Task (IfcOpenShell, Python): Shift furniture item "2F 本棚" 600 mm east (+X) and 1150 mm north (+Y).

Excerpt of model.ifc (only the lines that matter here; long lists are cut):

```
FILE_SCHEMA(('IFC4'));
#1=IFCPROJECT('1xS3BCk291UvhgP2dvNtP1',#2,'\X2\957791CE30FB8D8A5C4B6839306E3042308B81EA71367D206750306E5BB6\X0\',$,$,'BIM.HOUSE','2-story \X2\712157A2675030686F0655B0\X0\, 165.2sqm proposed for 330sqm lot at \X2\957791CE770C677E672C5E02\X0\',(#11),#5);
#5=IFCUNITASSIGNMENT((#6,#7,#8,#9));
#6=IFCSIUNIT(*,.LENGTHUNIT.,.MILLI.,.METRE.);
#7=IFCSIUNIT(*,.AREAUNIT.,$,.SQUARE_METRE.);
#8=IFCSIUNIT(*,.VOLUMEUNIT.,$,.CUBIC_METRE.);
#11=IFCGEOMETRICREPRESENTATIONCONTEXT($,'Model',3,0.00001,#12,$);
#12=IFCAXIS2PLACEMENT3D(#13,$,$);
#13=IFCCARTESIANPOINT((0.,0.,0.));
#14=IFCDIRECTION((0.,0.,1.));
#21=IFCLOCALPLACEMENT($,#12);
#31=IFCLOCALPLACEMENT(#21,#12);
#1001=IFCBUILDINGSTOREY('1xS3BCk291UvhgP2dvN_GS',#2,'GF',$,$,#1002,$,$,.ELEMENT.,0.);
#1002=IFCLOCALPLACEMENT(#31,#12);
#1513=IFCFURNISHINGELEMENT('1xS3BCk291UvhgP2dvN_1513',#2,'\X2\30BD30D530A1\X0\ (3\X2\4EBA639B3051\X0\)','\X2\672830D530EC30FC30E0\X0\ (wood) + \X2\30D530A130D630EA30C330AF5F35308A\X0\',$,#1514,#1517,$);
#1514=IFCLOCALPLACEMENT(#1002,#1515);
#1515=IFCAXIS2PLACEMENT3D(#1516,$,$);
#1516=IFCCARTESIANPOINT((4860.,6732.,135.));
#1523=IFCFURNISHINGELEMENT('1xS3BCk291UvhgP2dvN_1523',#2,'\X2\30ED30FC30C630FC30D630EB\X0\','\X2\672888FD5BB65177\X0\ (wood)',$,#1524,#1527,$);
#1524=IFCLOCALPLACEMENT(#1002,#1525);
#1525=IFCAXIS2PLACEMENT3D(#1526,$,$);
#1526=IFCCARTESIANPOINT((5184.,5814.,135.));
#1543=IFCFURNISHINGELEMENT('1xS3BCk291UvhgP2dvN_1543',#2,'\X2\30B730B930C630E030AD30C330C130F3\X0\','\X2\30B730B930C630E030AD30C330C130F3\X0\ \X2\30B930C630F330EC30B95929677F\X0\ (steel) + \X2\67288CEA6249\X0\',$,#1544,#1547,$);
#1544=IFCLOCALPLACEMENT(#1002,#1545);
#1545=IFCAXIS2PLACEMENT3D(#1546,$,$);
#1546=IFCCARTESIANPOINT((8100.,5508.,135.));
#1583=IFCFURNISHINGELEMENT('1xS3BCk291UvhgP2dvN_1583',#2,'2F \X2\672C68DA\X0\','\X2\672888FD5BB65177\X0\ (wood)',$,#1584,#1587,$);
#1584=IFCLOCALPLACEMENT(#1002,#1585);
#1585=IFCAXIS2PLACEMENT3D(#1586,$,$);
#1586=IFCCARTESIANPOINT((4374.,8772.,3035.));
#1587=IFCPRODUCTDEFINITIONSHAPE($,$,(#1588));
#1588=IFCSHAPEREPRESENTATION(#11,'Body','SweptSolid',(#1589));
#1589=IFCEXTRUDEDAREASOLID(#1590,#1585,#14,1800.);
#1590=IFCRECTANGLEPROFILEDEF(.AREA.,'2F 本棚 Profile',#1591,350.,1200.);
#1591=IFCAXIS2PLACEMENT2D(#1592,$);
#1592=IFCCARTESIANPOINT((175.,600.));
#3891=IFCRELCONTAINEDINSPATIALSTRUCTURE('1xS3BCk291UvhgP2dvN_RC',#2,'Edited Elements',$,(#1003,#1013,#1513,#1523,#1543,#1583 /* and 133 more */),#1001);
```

```python
import ifcopenshell
import ifcopenshell.api.geometry
import ifcopenshell.util.placement
import ifcopenshell.util.unit

model = ifcopenshell.open("model.ifc")
unit_scale = ifcopenshell.util.unit.calculate_unit_scale(model)

item = model.by_guid("1xS3BCk291UvhgP2dvN_1583")
matrix = ifcopenshell.util.placement.get_local_placement(item.ObjectPlacement)
matrix[0, 3] += 0.6 / unit_scale
matrix[1, 3] += 1.15 / unit_scale
ifcopenshell.api.geometry.edit_object_placement(model, product=item, matrix=matrix, is_si=False)

print(ifcopenshell.util.placement.get_local_placement(item.ObjectPlacement).round(3) + 0.0)

model.write("model_v2.ifc")
```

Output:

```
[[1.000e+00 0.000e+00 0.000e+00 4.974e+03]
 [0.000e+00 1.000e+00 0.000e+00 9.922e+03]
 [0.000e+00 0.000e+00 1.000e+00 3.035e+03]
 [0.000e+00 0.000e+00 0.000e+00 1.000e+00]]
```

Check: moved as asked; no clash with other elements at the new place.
